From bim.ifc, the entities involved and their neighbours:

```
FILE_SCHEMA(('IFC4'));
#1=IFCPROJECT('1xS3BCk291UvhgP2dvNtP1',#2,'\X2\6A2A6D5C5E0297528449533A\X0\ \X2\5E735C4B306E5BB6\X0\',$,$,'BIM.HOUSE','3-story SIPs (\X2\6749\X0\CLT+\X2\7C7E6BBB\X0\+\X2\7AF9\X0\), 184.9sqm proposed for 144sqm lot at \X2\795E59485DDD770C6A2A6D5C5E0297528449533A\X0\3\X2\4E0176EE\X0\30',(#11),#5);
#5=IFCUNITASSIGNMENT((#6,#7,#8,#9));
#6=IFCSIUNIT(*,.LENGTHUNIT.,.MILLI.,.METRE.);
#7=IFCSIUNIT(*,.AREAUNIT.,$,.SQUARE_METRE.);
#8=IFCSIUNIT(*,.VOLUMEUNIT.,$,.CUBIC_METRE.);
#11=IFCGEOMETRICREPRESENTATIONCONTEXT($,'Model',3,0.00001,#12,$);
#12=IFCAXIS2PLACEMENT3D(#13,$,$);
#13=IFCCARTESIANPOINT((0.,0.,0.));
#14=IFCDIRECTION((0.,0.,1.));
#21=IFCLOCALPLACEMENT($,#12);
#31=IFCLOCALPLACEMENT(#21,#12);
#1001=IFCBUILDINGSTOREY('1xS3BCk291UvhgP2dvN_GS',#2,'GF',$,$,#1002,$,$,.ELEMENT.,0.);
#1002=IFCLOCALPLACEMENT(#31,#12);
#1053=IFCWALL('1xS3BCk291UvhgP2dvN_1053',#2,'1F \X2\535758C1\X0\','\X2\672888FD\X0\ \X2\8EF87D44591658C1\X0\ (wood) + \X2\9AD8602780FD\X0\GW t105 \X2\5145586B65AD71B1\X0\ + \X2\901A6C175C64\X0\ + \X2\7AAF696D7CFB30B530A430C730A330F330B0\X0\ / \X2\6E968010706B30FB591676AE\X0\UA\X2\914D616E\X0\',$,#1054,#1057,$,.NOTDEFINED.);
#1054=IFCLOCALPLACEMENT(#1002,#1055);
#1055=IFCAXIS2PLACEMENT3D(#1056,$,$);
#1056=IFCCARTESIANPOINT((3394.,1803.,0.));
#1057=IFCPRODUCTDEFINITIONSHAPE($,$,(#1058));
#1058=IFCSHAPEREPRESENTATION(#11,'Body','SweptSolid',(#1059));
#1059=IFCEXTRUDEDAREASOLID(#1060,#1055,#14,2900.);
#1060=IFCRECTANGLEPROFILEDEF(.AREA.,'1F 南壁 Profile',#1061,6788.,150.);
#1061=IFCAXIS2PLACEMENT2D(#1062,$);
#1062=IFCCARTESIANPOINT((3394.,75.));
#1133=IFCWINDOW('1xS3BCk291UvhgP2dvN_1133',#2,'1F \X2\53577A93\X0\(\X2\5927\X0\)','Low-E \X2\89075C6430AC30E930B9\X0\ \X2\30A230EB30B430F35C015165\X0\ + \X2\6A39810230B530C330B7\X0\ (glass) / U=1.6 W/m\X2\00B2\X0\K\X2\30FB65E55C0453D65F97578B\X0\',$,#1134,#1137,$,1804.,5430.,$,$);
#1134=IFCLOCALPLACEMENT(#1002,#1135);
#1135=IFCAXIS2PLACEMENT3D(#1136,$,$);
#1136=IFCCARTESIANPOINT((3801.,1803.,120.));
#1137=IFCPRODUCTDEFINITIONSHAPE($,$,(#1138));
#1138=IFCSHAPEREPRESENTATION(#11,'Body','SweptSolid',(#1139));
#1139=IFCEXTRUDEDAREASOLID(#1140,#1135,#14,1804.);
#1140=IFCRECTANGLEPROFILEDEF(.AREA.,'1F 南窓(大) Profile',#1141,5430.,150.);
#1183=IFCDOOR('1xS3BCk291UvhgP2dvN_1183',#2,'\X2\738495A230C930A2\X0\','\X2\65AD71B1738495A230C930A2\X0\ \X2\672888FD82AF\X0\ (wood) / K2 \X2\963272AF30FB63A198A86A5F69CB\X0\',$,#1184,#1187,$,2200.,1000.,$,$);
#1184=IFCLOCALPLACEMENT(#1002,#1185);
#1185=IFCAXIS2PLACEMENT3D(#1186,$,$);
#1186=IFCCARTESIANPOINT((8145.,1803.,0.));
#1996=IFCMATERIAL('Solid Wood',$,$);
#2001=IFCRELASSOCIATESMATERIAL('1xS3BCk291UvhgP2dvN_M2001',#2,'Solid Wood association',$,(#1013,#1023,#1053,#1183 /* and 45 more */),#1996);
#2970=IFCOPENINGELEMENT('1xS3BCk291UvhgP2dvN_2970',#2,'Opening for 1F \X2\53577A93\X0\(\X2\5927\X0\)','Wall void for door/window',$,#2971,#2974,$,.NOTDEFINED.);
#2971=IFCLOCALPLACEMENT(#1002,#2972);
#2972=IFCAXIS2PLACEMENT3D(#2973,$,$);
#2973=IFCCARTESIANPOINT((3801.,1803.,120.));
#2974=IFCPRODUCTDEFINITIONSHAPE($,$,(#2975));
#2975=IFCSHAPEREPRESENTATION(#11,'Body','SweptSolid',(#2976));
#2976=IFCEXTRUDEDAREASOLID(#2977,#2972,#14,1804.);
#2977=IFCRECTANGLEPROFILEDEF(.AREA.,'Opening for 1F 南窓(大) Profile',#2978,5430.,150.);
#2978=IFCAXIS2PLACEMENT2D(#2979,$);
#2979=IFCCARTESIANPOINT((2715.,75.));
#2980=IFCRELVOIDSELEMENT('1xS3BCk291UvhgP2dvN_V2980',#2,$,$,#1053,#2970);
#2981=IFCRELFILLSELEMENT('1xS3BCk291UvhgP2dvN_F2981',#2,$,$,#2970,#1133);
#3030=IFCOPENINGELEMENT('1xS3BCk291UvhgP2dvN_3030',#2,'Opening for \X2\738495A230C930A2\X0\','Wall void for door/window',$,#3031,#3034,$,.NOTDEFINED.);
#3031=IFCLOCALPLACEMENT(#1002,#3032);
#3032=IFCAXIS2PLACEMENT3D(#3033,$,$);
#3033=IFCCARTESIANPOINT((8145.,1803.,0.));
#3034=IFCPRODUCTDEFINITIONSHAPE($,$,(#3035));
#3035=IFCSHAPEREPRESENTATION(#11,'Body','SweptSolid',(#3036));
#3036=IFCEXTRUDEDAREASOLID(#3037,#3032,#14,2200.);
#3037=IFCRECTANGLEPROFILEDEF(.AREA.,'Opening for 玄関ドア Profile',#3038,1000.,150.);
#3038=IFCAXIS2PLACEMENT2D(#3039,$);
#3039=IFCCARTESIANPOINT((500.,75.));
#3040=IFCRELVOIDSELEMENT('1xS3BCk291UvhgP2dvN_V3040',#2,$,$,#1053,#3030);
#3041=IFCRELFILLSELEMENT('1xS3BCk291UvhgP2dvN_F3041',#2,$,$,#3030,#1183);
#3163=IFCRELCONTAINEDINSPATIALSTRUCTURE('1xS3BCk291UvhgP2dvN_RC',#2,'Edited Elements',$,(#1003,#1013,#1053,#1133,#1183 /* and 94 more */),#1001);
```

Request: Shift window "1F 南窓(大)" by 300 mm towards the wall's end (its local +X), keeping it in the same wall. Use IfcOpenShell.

```python
import ifcopenshell
import ifcopenshell.api.geometry
import ifcopenshell.util.placement

model = ifcopenshell.open("bim.ifc")

window = model.by_guid("1xS3BCk291UvhgP2dvN_1133")
opening = window.FillsVoids[0].RelatingOpeningElement
wall = opening.VoidsElements[0].RelatingBuildingElement

wall_matrix = ifcopenshell.util.placement.get_local_placement(wall.ObjectPlacement)
shift = wall_matrix[:3, 0] * 300.0
before = ifcopenshell.util.placement.get_local_placement(window.ObjectPlacement)[:3, 3].copy()

# The window is not placed relative to its opening, so move both.
for product in (opening, window):
    matrix = ifcopenshell.util.placement.get_local_placement(product.ObjectPlacement)
    matrix[:3, 3] += shift
    ifcopenshell.api.geometry.edit_object_placement(model, product=product, matrix=matrix, is_si=False)

after = ifcopenshell.util.placement.get_local_placement(window.ObjectPlacement)[:3, 3]
print("window moved by", (after - before).round(3) + 0.0)

model.write("bim_updated.ifc")
```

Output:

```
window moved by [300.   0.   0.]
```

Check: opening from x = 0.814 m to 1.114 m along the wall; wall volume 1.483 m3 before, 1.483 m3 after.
